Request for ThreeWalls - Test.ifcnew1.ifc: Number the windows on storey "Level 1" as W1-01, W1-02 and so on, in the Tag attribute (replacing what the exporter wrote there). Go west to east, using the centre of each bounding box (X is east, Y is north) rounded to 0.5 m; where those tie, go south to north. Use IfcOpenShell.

First a look at what the model holds.

```python
import ifcopenshell
import ifcopenshell.util.element
import ifcopenshell.util.placement

model = ifcopenshell.open("ThreeWalls - Test.ifcnew1.ifc")
print(model.schema)
storey = next(s for s in model.by_type("IfcBuildingStorey") if s.Name == "Level 1")
windows = [e for e in ifcopenshell.util.element.get_decomposition(storey) if e.is_a("IfcWindow")]
for e in sorted(windows, key=lambda e: e.id()):
    origin = ifcopenshell.util.placement.get_local_placement(e.ObjectPlacement)[:3, 3]
    print(e.id(), e.Tag, e.Name, origin.round(2) + 0.0, sep=" | ")
```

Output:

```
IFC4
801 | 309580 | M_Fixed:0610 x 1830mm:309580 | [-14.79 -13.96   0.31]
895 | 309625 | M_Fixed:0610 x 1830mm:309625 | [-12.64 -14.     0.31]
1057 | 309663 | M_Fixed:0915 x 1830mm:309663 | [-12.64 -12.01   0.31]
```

```python
import ifcopenshell
import ifcopenshell.geom
import ifcopenshell.util.element
import ifcopenshell.util.shape

model = ifcopenshell.open("ThreeWalls - Test.ifcnew1.ifc")
settings = ifcopenshell.geom.settings()
settings.set("use-world-coords", True)


def centre(element):
    shape = ifcopenshell.geom.create_shape(settings, element)
    return ifcopenshell.util.shape.get_bbox_centroid(shape.geometry)


storey = next(s for s in model.by_type("IfcBuildingStorey") if s.Name == "Level 1")
windows = [e for e in ifcopenshell.util.element.get_decomposition(storey) if e.is_a("IfcWindow")]

# Insertion points can sit at a corner or the storey origin, so sort by the geometry (in metres).
centres = {e: centre(e) for e in windows}
windows.sort(key=lambda e: (round(centres[e][0] / 0.5), centres[e][1]))

for i, e in enumerate(windows, start=1):
    number = f"W1-{i:02d}"
    e.Tag = number
    print(e.id(), number)

model.write("ThreeWalls - Test.ifcnew1_v2.ifc")
```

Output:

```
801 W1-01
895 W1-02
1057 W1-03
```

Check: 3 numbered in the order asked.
